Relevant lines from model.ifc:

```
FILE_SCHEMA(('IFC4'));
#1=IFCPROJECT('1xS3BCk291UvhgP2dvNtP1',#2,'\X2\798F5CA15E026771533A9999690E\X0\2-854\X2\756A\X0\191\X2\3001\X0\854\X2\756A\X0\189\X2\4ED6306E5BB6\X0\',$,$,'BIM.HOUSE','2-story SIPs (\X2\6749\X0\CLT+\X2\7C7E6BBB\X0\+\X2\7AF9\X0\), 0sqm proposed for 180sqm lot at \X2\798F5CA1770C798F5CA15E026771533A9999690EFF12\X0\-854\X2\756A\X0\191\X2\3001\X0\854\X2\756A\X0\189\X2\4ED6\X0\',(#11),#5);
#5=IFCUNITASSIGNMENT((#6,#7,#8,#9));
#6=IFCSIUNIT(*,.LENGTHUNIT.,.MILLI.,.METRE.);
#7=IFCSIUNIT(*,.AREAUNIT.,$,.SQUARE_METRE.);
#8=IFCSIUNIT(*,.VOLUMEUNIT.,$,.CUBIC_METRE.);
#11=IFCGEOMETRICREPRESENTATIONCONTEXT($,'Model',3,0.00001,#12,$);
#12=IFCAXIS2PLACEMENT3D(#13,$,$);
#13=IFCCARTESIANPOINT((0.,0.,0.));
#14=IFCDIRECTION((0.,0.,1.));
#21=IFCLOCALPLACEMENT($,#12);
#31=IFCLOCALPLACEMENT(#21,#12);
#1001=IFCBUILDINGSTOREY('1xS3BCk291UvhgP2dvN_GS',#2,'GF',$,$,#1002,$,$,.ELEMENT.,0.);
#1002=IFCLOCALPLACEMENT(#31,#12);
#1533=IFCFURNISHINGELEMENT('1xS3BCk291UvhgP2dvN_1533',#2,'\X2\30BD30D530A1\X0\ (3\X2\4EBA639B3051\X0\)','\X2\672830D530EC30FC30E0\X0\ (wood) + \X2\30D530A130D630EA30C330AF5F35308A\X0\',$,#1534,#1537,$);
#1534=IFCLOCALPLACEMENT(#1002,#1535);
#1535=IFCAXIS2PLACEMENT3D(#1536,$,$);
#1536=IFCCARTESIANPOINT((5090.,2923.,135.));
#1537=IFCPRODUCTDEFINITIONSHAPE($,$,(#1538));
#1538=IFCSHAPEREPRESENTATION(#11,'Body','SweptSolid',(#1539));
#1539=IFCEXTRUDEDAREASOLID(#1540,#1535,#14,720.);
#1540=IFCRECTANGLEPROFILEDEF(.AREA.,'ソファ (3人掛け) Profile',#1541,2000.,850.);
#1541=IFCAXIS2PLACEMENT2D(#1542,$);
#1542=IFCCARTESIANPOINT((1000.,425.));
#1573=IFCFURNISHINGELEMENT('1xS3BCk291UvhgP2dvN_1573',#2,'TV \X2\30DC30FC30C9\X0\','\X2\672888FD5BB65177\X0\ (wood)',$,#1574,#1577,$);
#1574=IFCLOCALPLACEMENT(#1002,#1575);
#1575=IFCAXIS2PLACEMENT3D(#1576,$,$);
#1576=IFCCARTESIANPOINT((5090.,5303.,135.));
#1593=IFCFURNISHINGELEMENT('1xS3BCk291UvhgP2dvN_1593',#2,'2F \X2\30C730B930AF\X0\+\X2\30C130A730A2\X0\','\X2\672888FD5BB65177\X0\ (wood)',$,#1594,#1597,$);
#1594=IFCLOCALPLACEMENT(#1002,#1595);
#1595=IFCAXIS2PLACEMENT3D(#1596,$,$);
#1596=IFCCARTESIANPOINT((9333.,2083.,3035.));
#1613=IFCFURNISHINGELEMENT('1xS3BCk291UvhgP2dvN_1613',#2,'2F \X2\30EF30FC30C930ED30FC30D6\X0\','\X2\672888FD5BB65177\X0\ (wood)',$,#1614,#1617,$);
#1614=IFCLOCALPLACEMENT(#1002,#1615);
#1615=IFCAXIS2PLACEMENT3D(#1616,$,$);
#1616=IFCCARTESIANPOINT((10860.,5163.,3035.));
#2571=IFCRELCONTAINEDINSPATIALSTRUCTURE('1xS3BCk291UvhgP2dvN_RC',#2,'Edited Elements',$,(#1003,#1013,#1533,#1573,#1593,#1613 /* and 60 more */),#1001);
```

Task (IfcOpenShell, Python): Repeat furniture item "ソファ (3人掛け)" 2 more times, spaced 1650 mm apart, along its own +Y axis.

```python
import ifcopenshell
import ifcopenshell.api.geometry
import ifcopenshell.api.root
import ifcopenshell.util.element
import ifcopenshell.util.placement
import ifcopenshell.util.unit

model = ifcopenshell.open("model.ifc")
unit_scale = ifcopenshell.util.unit.calculate_unit_scale(model)


def reuse_history(source, copy):
    """copy_class also copies each property set's owner history, people and application; keep the originals."""
    for rel in copy.IsDefinedBy:
        if rel.is_a("IfcRelDefinesByProperties") and (history := rel.RelatingPropertyDefinition.OwnerHistory):
            rel.RelatingPropertyDefinition.OwnerHistory = source.OwnerHistory
            ifcopenshell.util.element.remove_deep2(model, history)


source = model.by_guid("1xS3BCk291UvhgP2dvN_1533")
base = ifcopenshell.util.placement.get_local_placement(source.ObjectPlacement)
step = base[:3, 1] * 1.65 / unit_scale

for i in range(1, 3):
    copy = ifcopenshell.api.root.copy_class(model, product=source)
    copy.Representation = ifcopenshell.util.element.copy_deep(
        model, source.Representation, exclude=["IfcGeometricRepresentationContext", "IfcRepresentationMap"]
    )
    reuse_history(source, copy)
    matrix = base.copy()
    matrix[:3, 3] += i * step
    print("added at", matrix[:3, 3].round(3) + 0.0)
    ifcopenshell.api.geometry.edit_object_placement(model, product=copy, matrix=matrix, is_si=False)

model.write("model_v2.ifc")
```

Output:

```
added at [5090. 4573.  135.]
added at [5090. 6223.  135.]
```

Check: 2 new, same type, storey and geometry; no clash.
